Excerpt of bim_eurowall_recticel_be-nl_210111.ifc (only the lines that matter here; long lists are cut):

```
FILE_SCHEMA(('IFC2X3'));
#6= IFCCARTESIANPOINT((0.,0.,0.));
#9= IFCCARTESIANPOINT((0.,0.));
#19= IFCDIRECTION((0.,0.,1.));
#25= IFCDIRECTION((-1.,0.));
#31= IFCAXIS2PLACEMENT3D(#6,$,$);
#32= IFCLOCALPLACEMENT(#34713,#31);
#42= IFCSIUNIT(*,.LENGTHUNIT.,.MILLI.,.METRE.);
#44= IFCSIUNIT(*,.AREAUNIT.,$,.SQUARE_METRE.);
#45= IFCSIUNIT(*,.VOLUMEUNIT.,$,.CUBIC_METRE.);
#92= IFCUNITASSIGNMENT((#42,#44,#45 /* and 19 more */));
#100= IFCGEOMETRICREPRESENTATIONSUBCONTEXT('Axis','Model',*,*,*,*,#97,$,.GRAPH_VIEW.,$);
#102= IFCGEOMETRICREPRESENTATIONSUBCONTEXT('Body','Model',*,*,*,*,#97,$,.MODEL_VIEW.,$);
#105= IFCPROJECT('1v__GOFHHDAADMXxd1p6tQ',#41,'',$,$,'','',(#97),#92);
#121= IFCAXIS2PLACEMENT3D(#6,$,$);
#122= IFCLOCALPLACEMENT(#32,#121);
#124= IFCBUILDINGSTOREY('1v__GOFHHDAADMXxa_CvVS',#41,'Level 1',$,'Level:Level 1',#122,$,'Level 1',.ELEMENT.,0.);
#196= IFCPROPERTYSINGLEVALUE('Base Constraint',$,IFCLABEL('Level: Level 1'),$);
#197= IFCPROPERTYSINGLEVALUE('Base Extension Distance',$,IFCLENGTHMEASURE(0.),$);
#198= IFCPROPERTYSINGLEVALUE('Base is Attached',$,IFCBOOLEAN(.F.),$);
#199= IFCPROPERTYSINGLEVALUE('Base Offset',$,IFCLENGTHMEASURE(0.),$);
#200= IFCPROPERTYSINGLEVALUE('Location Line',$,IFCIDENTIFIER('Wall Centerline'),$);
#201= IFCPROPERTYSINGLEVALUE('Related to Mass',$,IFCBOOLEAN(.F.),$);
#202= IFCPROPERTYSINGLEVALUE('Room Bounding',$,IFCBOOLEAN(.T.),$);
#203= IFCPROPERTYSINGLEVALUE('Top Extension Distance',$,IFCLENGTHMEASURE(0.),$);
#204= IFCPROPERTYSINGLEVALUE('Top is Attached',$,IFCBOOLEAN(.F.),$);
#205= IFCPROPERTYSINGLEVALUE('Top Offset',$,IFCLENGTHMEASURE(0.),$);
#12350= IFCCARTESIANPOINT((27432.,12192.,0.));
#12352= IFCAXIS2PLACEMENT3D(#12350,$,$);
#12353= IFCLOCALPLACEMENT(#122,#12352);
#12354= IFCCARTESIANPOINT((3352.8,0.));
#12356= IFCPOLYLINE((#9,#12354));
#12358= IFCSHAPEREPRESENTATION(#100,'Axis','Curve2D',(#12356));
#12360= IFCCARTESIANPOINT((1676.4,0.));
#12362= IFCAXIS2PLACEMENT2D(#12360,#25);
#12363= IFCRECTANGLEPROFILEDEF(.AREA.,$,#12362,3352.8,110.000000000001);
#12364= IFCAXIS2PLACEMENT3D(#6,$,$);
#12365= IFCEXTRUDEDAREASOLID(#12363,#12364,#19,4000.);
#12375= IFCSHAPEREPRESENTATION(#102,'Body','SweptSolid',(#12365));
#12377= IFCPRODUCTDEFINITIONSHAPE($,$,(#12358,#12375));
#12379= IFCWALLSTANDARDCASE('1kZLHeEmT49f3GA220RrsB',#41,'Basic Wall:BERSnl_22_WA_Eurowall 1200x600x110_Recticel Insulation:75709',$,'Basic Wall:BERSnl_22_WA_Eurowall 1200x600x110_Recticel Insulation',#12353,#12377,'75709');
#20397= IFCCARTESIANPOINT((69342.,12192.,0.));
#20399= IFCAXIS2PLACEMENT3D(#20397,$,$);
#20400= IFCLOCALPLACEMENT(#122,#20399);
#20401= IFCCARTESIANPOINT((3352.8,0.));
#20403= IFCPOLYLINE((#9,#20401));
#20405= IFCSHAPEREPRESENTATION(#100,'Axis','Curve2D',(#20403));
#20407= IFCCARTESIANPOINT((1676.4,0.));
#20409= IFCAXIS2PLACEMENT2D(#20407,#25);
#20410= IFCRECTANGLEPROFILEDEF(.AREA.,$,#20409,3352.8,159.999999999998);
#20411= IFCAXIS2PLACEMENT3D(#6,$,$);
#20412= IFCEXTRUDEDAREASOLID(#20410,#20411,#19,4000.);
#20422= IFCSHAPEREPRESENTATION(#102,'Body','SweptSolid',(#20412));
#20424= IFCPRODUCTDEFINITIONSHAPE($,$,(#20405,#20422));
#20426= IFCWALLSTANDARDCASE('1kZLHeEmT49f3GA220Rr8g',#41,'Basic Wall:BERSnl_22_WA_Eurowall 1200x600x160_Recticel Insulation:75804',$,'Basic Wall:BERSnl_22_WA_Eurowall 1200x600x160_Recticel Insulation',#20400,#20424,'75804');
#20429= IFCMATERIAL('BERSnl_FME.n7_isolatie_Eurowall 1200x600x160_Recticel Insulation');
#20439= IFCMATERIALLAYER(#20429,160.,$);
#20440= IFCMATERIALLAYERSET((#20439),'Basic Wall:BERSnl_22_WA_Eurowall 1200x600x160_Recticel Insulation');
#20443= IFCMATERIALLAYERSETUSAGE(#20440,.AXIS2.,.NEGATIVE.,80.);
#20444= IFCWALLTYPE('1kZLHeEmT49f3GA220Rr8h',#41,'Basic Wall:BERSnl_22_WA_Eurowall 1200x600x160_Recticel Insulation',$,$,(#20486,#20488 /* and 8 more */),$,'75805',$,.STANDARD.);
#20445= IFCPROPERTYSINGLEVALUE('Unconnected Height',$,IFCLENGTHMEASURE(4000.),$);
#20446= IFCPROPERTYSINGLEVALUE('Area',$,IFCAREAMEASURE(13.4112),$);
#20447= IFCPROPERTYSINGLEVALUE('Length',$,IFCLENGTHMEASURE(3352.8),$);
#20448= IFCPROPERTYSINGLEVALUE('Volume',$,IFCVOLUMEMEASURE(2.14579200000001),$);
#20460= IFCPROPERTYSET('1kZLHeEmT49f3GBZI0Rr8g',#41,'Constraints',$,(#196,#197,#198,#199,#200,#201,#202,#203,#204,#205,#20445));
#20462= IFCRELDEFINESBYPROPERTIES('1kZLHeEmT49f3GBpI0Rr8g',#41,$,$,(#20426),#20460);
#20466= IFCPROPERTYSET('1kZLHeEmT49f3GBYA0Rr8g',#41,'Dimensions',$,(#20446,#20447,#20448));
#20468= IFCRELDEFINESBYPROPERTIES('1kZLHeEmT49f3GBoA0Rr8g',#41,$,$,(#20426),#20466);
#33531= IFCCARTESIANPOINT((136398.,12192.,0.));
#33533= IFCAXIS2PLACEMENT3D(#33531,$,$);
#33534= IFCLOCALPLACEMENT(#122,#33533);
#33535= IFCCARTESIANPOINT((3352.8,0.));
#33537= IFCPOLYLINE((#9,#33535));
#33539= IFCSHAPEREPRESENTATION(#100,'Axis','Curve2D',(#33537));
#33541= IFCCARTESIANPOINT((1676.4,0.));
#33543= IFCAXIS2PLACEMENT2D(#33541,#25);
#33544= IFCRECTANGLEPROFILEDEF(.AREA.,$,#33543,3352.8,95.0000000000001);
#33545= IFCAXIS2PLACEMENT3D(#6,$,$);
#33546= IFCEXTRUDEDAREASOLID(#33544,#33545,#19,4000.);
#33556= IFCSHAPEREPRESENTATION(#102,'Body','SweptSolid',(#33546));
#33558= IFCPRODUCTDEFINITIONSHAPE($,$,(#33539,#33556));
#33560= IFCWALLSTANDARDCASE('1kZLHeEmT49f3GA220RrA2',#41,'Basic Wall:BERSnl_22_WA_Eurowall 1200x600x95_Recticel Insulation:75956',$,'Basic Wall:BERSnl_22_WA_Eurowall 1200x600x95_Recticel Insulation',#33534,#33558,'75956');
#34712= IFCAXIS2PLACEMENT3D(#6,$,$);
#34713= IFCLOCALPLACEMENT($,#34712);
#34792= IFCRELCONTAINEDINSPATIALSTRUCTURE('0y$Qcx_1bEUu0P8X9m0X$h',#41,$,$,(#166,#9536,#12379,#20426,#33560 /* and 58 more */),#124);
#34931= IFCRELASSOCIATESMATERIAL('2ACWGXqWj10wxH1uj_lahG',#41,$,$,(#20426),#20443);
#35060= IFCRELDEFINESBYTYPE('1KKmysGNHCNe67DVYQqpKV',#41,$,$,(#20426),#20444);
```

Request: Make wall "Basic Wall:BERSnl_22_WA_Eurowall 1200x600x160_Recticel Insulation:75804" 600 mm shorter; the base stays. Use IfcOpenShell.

```python
import ifcopenshell
import ifcopenshell.api.pset
import ifcopenshell.geom
import ifcopenshell.util.element
import ifcopenshell.util.representation
import ifcopenshell.util.shape
import ifcopenshell.util.unit

model = ifcopenshell.open("bim_eurowall_recticel_be-nl_210111.ifc")
area_scale = ifcopenshell.util.unit.calculate_unit_scale(model, "AREAUNIT")
volume_scale = ifcopenshell.util.unit.calculate_unit_scale(model, "VOLUMEUNIT")
settings = ifcopenshell.geom.settings()


def volume(element):
    """Net volume in cubic metres, openings subtracted."""
    shape = ifcopenshell.geom.create_shape(settings, element)
    return ifcopenshell.util.shape.get_volume(shape.geometry)


wall = model.by_guid("1kZLHeEmT49f3GA220Rr8g")
before = volume(wall)

body = ifcopenshell.util.representation.get_representation(wall, "Model", "Body")
solid = body.Items[0]
old_height = solid.Depth
solid.Depth -= 600.0
after = volume(wall)
thickness = 0.16  # wall thickness in metres

# Update the stored height, areas and volumes.
pset = model.by_id(ifcopenshell.util.element.get_pset(wall, "Constraints", should_inherit=False)["id"])
ifcopenshell.api.pset.edit_pset(model, pset=pset, properties={
    "Unconnected Height": model.create_entity("IfcLengthMeasure", solid.Depth),
})
pset = model.by_id(ifcopenshell.util.element.get_pset(wall, "Dimensions", should_inherit=False)["id"])
ifcopenshell.api.pset.edit_pset(model, pset=pset, properties={
    "Area": model.create_entity("IfcAreaMeasure", after / thickness / area_scale),
    "Volume": model.create_entity("IfcVolumeMeasure", after / volume_scale),
})

print(f"height {old_height:g} -> {solid.Depth:g}, volume {before:.3f} -> {after:.3f} m3")

model.write("bim_eurowall_recticel_be-nl_210111_updated.ifc")
```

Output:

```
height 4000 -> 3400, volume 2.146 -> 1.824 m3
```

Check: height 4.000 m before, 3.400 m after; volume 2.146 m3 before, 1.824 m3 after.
